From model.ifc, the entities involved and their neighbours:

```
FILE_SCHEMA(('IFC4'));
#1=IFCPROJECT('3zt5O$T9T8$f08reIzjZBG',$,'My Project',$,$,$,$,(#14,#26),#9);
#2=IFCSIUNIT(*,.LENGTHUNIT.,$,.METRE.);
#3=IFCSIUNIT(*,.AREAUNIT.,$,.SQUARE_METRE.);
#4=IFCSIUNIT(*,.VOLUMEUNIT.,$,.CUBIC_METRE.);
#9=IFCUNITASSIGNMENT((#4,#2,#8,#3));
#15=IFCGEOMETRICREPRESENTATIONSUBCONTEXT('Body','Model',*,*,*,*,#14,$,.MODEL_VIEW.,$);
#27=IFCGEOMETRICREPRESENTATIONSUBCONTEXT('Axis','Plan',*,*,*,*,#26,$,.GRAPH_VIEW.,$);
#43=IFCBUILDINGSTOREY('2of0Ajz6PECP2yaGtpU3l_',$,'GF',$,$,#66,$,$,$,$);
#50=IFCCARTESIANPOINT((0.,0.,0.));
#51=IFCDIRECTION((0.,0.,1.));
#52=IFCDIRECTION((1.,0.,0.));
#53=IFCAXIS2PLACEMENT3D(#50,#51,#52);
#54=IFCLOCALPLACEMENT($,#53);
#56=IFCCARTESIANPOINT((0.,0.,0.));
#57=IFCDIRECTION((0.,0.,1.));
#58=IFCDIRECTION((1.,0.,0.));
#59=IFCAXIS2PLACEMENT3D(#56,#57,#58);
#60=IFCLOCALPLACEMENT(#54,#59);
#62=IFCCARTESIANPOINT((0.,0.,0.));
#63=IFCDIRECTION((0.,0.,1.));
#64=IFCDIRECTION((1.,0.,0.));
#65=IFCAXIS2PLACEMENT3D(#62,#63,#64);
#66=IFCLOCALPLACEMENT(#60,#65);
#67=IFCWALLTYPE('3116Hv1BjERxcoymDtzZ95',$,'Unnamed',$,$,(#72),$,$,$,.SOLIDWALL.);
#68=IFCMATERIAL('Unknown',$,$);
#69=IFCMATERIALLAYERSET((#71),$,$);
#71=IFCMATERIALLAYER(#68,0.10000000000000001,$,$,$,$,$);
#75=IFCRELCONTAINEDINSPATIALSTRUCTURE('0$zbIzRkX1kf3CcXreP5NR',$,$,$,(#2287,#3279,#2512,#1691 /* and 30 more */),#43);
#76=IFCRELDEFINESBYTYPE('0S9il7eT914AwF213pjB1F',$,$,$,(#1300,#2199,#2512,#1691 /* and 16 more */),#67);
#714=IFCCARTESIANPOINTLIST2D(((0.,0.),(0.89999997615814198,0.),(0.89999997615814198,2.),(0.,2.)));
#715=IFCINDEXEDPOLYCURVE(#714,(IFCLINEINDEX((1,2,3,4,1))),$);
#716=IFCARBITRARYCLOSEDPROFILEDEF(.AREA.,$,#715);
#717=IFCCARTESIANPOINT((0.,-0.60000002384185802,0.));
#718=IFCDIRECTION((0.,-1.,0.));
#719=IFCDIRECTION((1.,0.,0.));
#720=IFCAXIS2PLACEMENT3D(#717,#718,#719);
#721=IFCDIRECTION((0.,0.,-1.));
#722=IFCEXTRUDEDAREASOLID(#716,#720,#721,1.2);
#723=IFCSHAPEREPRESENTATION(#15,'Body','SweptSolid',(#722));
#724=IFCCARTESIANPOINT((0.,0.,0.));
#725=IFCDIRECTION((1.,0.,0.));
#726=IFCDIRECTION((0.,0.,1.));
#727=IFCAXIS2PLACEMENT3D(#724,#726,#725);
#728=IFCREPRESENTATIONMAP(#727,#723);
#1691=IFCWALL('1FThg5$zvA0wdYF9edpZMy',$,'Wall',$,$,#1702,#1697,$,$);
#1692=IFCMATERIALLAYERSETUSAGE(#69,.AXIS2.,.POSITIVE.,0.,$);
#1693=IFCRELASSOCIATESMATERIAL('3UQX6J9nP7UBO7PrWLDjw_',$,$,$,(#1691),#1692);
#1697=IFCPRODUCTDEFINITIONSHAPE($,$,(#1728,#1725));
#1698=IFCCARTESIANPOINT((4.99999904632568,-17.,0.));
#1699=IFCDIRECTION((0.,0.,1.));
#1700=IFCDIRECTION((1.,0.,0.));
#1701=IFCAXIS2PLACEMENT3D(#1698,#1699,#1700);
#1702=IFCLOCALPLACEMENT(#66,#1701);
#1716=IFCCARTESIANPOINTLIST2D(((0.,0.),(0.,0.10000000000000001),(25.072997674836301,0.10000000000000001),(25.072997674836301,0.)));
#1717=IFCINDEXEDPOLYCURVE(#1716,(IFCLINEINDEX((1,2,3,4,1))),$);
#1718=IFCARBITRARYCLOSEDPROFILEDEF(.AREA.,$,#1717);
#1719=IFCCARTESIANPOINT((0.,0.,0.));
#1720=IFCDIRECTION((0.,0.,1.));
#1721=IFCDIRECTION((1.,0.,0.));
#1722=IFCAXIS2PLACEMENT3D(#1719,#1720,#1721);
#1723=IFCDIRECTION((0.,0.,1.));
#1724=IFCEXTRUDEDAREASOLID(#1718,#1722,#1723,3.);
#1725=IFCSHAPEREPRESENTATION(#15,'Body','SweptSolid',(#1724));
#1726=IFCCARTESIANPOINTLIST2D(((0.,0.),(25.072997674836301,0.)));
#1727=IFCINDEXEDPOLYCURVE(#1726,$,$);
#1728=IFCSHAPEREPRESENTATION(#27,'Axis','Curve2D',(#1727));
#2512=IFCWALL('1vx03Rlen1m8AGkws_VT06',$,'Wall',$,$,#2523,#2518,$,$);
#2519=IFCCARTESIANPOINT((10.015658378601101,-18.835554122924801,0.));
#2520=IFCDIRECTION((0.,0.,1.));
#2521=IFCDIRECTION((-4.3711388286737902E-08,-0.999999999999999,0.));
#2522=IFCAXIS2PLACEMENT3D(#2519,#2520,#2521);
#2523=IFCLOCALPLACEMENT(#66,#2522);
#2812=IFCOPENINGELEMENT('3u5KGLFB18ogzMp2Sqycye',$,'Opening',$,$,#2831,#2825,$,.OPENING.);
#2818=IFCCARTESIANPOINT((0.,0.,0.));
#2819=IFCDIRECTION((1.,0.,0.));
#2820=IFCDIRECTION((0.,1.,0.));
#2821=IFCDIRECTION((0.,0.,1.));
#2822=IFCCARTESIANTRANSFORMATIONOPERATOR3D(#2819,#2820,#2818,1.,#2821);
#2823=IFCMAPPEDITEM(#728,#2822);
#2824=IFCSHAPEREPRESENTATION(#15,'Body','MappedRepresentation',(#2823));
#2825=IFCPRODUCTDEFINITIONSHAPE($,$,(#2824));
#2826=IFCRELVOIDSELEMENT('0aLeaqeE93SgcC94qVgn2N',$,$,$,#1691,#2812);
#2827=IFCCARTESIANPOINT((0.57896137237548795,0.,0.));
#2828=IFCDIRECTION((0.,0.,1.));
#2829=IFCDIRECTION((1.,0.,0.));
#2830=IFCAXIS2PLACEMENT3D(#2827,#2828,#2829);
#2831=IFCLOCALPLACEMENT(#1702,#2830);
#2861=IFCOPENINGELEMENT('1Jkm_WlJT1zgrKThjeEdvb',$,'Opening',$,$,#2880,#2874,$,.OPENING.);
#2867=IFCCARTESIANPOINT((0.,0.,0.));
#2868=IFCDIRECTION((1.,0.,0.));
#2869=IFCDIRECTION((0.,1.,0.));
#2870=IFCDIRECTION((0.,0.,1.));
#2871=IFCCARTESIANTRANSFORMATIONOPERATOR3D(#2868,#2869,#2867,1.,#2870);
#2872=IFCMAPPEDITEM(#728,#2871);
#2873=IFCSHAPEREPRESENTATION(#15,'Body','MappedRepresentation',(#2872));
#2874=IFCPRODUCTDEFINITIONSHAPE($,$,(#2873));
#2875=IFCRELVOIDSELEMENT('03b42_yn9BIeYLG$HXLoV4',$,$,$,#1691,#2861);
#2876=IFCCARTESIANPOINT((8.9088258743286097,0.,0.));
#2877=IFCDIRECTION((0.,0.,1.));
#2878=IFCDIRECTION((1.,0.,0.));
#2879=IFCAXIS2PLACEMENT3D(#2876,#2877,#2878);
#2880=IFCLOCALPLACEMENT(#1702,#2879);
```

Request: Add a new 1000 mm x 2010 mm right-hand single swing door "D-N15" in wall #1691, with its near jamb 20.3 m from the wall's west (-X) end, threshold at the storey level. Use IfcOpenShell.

```python
import numpy as np
import ifcopenshell
import ifcopenshell.api.feature
import ifcopenshell.api.geometry
import ifcopenshell.api.root
import ifcopenshell.api.spatial
import ifcopenshell.geom
import ifcopenshell.util.element
import ifcopenshell.util.placement
import ifcopenshell.util.representation
import ifcopenshell.util.shape
import ifcopenshell.util.unit

model = ifcopenshell.open("model.ifc")
unit_scale = ifcopenshell.util.unit.calculate_unit_scale(model)
settings = ifcopenshell.geom.settings()


def volume(element):
    """Net volume in cubic metres, openings subtracted."""
    shape = ifcopenshell.geom.create_shape(settings, element)
    return ifcopenshell.util.shape.get_volume(shape.geometry)


wall = model.by_guid("1FThg5$zvA0wdYF9edpZMy")
storey = ifcopenshell.util.element.get_container(wall, ifc_class="IfcBuildingStorey")
context = ifcopenshell.util.representation.get_context(model, "Model", "Body", "MODEL_VIEW")
before = volume(wall)

width, height, from_end, sill = 1, 2.01, 20.3, 0.0  # metres

# The wall runs along its own X axis, and the end named is its -X end.
wall_shape = ifcopenshell.geom.create_shape(settings, wall)
x, y, z = ifcopenshell.util.shape.get_vertices(wall_shape.geometry).T
start = x.min() + from_end
face, thickness = float(y.min()), float(y.max() - y.min())
wall_matrix = ifcopenshell.util.placement.get_local_placement(wall.ObjectPlacement)
level = ifcopenshell.util.placement.get_local_placement(storey.ObjectPlacement)[2, 3]


def in_wall(x, y):
    """Placement at x, y metres in the wall's axes, at sill height."""
    matrix = wall_matrix.copy()
    matrix[:, 3] = wall_matrix @ np.array([x / unit_scale, y / unit_scale, 0.0, 1.0])
    matrix[2, 3] = level + sill / unit_scale
    return matrix


# Opening: a box that overshoots both wall faces by 50 mm.
opening = ifcopenshell.api.root.create_entity(model, ifc_class="IfcOpeningElement", predefined_type="OPENING")
box = ifcopenshell.api.geometry.add_wall_representation(
    model, context=context, length=width, height=height, thickness=thickness + 0.1
)
ifcopenshell.api.geometry.assign_representation(model, product=opening, representation=box)
ifcopenshell.api.geometry.edit_object_placement(model, product=opening, matrix=in_wall(start, face - 0.05), is_si=False)
ifcopenshell.api.feature.add_feature(model, feature=opening, element=wall)

door = ifcopenshell.api.root.create_entity(model, ifc_class="IfcDoor", name="D-N15", predefined_type="DOOR")
door.OverallWidth, door.OverallHeight = width / unit_scale, height / unit_scale
door.OperationType = "SINGLE_SWING_RIGHT"
body = ifcopenshell.api.geometry.add_door_representation(
    model,
    context=context,
    overall_width=door.OverallWidth,
    overall_height=door.OverallHeight,
    operation_type="SINGLE_SWING_RIGHT",
    lining_properties={"LiningDepth": thickness / unit_scale, "ThresholdDepth": thickness / unit_scale},
)
ifcopenshell.api.geometry.assign_representation(model, product=door, representation=body)
ifcopenshell.api.spatial.assign_container(model, products=[door], relating_structure=storey)
ifcopenshell.api.feature.add_filling(model, opening=opening, element=door)

# The lining spans the wall, so the door starts at the wall face.
ifcopenshell.api.geometry.edit_object_placement(model, product=door, matrix=in_wall(start, face), is_si=False)

after = volume(wall)

print(f"wall volume {before:.3f} -> {after:.3f} m3")

model.write("model_rev.ifc")
```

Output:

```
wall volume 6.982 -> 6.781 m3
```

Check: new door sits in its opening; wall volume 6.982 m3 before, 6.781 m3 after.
